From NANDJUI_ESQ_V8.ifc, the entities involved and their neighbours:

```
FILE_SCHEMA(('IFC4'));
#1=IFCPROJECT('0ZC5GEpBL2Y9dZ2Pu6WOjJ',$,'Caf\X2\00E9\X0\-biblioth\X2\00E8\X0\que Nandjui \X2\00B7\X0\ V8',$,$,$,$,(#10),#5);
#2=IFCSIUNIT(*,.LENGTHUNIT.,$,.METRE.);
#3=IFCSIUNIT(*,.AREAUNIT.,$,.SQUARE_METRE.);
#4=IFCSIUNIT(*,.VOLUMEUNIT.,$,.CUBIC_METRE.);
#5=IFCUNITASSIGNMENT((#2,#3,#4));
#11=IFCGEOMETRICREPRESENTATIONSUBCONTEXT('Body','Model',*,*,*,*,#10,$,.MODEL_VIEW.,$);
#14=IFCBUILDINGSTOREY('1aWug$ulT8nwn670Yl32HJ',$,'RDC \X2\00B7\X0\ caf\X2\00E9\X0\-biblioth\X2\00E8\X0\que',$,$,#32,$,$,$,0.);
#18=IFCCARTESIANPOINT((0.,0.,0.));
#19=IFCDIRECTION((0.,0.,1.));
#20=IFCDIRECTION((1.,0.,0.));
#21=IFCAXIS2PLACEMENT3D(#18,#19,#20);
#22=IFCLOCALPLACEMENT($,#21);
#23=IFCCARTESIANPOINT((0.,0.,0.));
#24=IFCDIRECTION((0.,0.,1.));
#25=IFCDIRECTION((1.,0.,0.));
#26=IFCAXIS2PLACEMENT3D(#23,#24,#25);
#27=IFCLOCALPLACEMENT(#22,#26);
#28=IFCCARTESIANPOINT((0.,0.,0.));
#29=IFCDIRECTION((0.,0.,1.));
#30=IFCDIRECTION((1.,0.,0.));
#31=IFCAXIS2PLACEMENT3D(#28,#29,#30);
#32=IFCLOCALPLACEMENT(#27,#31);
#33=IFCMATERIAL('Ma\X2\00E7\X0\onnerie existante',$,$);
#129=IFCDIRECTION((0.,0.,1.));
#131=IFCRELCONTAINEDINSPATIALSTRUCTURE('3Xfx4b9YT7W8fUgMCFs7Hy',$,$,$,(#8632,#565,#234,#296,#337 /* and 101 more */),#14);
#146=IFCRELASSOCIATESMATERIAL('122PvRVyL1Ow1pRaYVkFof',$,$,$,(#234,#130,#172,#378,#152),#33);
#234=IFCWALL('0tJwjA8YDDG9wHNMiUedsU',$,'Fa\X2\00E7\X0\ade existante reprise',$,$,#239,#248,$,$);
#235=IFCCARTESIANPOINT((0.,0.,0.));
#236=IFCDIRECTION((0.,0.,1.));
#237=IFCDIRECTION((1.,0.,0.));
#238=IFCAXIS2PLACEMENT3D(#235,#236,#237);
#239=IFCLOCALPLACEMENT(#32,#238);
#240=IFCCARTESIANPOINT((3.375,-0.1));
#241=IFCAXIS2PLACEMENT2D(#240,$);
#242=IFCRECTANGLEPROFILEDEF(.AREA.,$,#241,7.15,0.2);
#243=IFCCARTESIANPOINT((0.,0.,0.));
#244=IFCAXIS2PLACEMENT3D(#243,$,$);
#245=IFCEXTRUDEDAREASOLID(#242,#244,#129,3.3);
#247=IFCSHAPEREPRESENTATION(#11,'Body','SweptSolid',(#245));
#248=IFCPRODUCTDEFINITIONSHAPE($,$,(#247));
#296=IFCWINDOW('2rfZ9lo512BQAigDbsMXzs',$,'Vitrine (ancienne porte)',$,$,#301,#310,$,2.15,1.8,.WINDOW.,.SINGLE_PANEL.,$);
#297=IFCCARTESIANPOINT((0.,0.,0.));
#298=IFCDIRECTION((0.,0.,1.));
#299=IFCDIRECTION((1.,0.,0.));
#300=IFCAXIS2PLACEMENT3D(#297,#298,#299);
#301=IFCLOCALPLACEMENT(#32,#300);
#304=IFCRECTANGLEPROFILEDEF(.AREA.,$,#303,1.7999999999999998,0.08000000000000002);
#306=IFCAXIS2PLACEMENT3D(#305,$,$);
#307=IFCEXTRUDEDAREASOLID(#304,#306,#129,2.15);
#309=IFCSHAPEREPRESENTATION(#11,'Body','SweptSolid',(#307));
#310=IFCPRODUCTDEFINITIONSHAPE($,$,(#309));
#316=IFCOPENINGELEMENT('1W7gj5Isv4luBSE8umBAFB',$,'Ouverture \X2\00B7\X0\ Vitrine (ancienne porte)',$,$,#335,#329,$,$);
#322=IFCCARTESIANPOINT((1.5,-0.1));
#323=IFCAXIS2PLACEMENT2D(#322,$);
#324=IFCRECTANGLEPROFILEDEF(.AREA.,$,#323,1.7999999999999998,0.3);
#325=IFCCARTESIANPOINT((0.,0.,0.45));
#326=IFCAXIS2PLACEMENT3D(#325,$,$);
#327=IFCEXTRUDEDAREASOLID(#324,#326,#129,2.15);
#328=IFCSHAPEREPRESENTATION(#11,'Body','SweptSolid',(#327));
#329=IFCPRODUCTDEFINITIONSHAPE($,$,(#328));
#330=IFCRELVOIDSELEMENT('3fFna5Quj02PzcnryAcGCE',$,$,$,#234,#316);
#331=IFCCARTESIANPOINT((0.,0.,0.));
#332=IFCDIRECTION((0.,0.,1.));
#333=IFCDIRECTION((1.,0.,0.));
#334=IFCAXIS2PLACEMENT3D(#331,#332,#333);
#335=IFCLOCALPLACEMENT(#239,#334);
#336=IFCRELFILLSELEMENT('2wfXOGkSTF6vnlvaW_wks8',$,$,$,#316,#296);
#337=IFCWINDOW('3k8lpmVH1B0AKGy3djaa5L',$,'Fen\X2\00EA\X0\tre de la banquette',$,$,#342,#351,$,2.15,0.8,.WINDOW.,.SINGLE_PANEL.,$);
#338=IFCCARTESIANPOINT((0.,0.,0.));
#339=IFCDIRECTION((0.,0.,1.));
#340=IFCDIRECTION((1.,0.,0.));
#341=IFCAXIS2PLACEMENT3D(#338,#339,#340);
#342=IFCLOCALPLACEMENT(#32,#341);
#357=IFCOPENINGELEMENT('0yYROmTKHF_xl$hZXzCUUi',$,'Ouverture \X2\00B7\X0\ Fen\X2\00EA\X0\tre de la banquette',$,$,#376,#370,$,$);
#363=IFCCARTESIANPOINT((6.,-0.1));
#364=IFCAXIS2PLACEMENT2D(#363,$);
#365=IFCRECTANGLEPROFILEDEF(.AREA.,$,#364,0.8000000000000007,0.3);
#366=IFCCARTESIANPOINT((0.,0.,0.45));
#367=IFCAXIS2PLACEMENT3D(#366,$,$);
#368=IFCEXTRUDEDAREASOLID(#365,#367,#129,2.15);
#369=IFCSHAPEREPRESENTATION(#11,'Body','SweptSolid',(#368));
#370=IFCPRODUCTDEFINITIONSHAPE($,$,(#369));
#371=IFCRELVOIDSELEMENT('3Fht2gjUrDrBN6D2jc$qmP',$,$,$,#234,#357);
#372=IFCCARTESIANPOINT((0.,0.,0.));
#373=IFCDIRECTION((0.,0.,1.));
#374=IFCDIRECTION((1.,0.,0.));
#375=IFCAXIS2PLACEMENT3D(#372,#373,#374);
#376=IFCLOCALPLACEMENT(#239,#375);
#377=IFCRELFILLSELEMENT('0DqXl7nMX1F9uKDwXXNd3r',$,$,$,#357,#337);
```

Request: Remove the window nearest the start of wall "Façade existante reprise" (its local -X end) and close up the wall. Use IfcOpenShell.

```python
import ifcopenshell
import ifcopenshell.api.feature
import ifcopenshell.api.root
import ifcopenshell.geom
import ifcopenshell.util.shape

model = ifcopenshell.open("NANDJUI_ESQ_V8.ifc")
settings = ifcopenshell.geom.settings()


def volume(element):
    """Net volume in cubic metres, openings subtracted."""
    shape = ifcopenshell.geom.create_shape(settings, element)
    return ifcopenshell.util.shape.get_volume(shape.geometry)


window = model.by_guid("2rfZ9lo512BQAigDbsMXzs")
opening = window.FillsVoids[0].RelatingOpeningElement
wall = opening.VoidsElements[0].RelatingBuildingElement
before = volume(wall)

ifcopenshell.api.root.remove_product(model, product=window)
ifcopenshell.api.feature.remove_feature(model, feature=opening)

after = volume(wall)

print(f"wall volume {before:.3f} -> {after:.3f} m3")

model.write("NANDJUI_ESQ_V8_rev.ifc")
```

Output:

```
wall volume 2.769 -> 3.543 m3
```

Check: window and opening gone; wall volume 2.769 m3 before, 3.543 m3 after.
